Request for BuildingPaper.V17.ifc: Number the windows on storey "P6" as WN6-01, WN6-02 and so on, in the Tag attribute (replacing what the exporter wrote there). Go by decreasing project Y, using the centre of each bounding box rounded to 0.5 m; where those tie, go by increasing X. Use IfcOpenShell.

First a look at what the model holds.

```python
import ifcopenshell
import ifcopenshell.util.element
import ifcopenshell.util.placement

model = ifcopenshell.open("BuildingPaper.V17.ifc")
print(model.schema)
storey = next(s for s in model.by_type("IfcBuildingStorey") if s.Name == "P6")
windows = [e for e in ifcopenshell.util.element.get_decomposition(storey) if e.is_a("IfcWindow")]
for e in sorted(windows, key=lambda e: e.id()):
    origin = ifcopenshell.util.placement.get_local_placement(e.ObjectPlacement)[:3, 3]
    print(e.id(), e.Tag, e.Name, origin.round(2) + 0.0, sep=" | ")
```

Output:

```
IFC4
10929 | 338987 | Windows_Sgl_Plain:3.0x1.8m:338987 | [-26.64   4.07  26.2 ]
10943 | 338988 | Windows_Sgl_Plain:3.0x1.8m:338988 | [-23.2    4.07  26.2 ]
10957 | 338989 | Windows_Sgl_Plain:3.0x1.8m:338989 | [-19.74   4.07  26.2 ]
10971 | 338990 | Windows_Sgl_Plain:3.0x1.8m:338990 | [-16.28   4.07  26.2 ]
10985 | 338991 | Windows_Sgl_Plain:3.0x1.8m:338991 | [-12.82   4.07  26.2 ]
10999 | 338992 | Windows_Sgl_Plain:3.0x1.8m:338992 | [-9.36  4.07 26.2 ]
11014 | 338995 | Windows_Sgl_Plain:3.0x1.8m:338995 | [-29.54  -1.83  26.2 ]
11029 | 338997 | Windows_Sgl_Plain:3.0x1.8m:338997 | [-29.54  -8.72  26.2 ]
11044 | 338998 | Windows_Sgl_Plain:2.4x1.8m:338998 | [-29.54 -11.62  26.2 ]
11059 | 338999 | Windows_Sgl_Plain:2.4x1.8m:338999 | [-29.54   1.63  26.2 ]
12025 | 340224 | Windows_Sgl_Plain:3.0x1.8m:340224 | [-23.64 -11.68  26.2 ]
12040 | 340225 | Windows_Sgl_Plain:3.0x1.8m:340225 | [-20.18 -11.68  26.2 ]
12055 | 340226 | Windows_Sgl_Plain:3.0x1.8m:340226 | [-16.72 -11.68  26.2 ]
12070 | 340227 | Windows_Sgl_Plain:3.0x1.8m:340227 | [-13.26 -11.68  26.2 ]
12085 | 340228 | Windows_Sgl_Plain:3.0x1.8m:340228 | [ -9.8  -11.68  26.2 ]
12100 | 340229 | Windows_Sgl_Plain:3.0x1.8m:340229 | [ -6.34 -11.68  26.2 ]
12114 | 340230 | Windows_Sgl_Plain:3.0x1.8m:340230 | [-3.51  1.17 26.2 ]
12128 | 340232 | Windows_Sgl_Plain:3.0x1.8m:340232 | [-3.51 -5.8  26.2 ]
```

```python
import ifcopenshell
import ifcopenshell.geom
import ifcopenshell.util.element
import ifcopenshell.util.shape

model = ifcopenshell.open("BuildingPaper.V17.ifc")
settings = ifcopenshell.geom.settings()
settings.set("use-world-coords", True)


def centre(element):
    shape = ifcopenshell.geom.create_shape(settings, element)
    return ifcopenshell.util.shape.get_bbox_centroid(shape.geometry)


storey = next(s for s in model.by_type("IfcBuildingStorey") if s.Name == "P6")
windows = [e for e in ifcopenshell.util.element.get_decomposition(storey) if e.is_a("IfcWindow")]

# Insertion points can sit at a corner or the storey origin, so sort by the geometry (in metres).
centres = {e: centre(e) for e in windows}
windows.sort(key=lambda e: (-round(centres[e][1] / 0.5), centres[e][0]))

for i, e in enumerate(windows, start=1):
    number = f"WN6-{i:02d}"
    e.Tag = number
    print(e.id(), number)

model.write("BuildingPaper.V17_updated.ifc")
```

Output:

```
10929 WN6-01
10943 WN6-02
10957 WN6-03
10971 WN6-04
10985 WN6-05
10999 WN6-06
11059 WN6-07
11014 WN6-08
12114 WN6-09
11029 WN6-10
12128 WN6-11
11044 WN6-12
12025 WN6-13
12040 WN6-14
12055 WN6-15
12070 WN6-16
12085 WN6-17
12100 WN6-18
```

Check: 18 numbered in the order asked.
